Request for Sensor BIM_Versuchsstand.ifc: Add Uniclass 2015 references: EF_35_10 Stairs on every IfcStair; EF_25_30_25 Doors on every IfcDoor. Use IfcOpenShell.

First a look at what the model holds.

```python
import ifcopenshell

model = ifcopenshell.open("Sensor BIM_Versuchsstand.ifc")
print(model.schema)
print("classifications:", [c.Name for c in model.by_type("IfcClassification")])
for ifc_class in ("IfcDoor", "IfcRoof", "IfcStair", "IfcWall", "IfcWindow"):
    print(ifc_class, len(model.by_type(ifc_class)))
```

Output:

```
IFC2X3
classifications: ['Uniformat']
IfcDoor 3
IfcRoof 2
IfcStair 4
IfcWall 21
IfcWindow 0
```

```python
import ifcopenshell
import ifcopenshell.api.classification

model = ifcopenshell.open("Sensor BIM_Versuchsstand.ifc")

# IFC2X3 requires Source and Edition and has no link from the project to the system.
system = model.create_entity("IfcClassification", Source="NBS", Edition="2015", Name="Uniclass 2015")

codes = {
    "IfcStair": ("EF_35_10", "Stairs"),
    "IfcDoor": ("EF_25_30_25", "Doors"),
}
for ifc_class, (code, name) in codes.items():
    products = model.by_type(ifc_class)
    ifcopenshell.api.classification.add_reference(
        model, products=products, classification=system, identification=code, name=name
    )
    print(code, len(products))

model.write("Sensor BIM_Versuchsstand_edited.ifc")
```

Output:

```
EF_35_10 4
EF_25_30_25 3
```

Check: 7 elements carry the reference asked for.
